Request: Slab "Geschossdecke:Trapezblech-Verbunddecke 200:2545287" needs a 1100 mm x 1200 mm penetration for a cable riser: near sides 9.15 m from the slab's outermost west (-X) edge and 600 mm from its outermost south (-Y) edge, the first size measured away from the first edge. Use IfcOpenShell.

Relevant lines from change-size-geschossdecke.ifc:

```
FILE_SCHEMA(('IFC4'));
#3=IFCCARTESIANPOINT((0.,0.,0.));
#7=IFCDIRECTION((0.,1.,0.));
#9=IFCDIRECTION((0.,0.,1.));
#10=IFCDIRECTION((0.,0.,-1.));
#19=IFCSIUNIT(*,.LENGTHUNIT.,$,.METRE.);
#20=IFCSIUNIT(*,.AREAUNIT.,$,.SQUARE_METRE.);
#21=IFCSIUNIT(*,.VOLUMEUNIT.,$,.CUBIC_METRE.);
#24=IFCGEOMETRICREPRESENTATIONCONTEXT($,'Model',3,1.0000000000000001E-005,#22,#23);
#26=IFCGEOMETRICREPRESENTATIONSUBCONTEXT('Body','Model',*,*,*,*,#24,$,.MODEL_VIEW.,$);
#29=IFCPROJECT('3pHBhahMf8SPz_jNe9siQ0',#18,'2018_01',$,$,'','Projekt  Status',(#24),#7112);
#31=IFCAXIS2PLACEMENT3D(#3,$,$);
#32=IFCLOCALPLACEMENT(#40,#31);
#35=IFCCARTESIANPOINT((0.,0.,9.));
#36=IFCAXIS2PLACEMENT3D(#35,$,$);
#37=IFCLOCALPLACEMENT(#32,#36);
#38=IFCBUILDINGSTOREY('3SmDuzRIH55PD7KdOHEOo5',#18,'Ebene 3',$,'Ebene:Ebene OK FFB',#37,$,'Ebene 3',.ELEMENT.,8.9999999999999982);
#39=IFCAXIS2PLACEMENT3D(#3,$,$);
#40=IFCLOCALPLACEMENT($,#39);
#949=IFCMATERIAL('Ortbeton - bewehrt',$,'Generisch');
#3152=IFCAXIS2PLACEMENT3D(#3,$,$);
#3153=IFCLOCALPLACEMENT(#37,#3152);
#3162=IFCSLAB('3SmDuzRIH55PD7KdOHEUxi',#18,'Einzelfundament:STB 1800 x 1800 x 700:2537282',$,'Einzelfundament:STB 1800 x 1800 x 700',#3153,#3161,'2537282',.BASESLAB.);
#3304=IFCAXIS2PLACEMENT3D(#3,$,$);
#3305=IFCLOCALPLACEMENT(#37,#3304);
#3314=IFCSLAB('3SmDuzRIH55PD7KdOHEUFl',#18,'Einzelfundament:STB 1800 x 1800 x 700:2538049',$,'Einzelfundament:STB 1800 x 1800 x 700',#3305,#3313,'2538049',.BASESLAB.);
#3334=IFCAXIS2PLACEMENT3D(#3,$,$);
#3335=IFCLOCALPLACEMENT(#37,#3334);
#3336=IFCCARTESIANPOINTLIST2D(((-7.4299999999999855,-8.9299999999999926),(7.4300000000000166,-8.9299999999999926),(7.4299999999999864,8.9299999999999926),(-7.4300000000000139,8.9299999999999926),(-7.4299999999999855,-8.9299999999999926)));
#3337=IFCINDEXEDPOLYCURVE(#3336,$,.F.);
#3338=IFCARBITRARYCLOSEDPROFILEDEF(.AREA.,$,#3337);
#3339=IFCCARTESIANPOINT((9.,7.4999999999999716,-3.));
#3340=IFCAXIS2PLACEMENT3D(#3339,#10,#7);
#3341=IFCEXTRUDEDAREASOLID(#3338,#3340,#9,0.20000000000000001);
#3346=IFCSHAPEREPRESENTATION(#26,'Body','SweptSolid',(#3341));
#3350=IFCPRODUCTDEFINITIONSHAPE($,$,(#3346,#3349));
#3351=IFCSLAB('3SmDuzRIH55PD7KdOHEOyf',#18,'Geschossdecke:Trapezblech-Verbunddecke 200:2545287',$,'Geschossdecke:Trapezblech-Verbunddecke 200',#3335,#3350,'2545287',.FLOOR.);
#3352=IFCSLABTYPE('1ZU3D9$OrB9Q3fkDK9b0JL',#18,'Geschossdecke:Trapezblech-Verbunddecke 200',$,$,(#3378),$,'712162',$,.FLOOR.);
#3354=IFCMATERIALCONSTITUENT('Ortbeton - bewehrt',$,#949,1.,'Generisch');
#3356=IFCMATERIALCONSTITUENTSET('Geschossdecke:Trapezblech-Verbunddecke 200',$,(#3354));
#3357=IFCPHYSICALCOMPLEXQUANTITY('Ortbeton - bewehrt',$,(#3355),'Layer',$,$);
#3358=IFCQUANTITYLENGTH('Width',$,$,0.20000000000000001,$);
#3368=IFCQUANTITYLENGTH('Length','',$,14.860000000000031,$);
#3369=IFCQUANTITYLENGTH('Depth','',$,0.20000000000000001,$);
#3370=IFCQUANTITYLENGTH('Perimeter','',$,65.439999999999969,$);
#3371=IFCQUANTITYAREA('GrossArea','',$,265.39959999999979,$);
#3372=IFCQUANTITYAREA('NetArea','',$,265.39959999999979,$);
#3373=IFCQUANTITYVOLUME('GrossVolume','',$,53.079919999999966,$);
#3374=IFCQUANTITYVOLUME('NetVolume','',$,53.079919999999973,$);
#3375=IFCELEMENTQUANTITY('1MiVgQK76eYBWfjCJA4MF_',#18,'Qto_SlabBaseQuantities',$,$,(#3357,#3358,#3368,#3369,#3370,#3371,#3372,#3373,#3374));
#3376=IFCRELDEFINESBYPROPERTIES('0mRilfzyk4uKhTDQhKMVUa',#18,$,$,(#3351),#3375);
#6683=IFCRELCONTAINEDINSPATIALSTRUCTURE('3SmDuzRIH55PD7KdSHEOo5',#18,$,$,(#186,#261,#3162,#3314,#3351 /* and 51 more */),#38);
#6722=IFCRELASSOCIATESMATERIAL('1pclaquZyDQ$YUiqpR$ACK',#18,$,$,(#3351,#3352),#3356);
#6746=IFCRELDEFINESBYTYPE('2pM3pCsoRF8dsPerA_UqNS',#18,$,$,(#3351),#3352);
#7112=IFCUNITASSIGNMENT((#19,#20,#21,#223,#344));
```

```python
import numpy as np
import ifcopenshell
import ifcopenshell.api.feature
import ifcopenshell.api.geometry
import ifcopenshell.api.pset
import ifcopenshell.api.root
import ifcopenshell.geom
import ifcopenshell.util.element
import ifcopenshell.util.placement
import ifcopenshell.util.representation
import ifcopenshell.util.shape
import ifcopenshell.util.unit

model = ifcopenshell.open("change-size-geschossdecke.ifc")
unit_scale = ifcopenshell.util.unit.calculate_unit_scale(model)
area_scale = ifcopenshell.util.unit.calculate_unit_scale(model, "AREAUNIT")
volume_scale = ifcopenshell.util.unit.calculate_unit_scale(model, "VOLUMEUNIT")
settings = ifcopenshell.geom.settings()


def volume(element):
    """Net volume in cubic metres, openings subtracted."""
    shape = ifcopenshell.geom.create_shape(settings, element)
    return ifcopenshell.util.shape.get_volume(shape.geometry)


slab = model.by_guid("3SmDuzRIH55PD7KdOHEOyf")
before = volume(slab)

# Extent in the slab's own axes, in metres. The edges named are its -X and -Y sides.
slab_shape = ifcopenshell.geom.create_shape(settings, slab)
vertices = ifcopenshell.util.shape.get_vertices(slab_shape.geometry)
x_min, y_min, bottom = vertices.min(axis=0)
top = vertices[:, 2].max()

opening = ifcopenshell.api.root.create_entity(model, ifc_class="IfcOpeningElement", name="Cable riser opening", predefined_type="OPENING")
context = ifcopenshell.util.representation.get_context(model, "Model", "Body", "MODEL_VIEW")
width, depth = 1.1, 1.2
outline = [(0.0, 0.0), (width, 0.0), (width, depth), (0.0, depth), (0.0, 0.0)]
# Overshoot both faces by 50 mm so the cut is clean.
shape = ifcopenshell.api.geometry.add_slab_representation(
    model, context=context, depth=top - bottom + 0.1, polyline=outline
)
ifcopenshell.api.geometry.assign_representation(model, product=opening, representation=shape)

matrix = ifcopenshell.util.placement.get_local_placement(slab.ObjectPlacement)
matrix[:, 3] = matrix @ np.append(np.array([x_min + 9.15, y_min + 0.6, bottom - 0.05]) / unit_scale, 1.0)
ifcopenshell.api.geometry.edit_object_placement(model, product=opening, matrix=matrix, is_si=False)
ifcopenshell.api.feature.add_feature(model, feature=opening, element=slab)

after = volume(slab)

# Update the slab's stored quantities.
qto = model.by_id(ifcopenshell.util.element.get_pset(slab, "Qto_SlabBaseQuantities", should_inherit=False)["id"])
ifcopenshell.api.pset.edit_qto(model, qto=qto, properties={
    "NetArea": after / (top - bottom) / area_scale,
    "NetVolume": after / volume_scale,
})

print(f"slab volume {before:.3f} -> {after:.3f} m3")

model.write("change-size-geschossdecke_rev.ifc")
```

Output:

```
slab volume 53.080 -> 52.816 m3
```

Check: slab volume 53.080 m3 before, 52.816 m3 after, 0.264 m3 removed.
